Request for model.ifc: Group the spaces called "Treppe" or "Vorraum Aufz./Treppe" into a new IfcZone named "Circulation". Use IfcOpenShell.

First a look at what the model holds.

```python
import ifcopenshell

model = ifcopenshell.open("model.ifc")
print(model.schema)
seen = {}
for space in model.by_type("IfcSpace"):
    seen[space.LongName] = seen.get(space.LongName, 0) + 1
for name, count in sorted(seen.items(), key=str):
    print(count, "x", name)
print("zones:", [z.Name for z in model.by_type("IfcZone")][:20])
```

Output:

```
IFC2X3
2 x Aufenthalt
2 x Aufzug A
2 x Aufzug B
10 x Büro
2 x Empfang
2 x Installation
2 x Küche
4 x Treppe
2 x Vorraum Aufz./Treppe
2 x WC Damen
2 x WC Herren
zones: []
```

```python
import ifcopenshell
import ifcopenshell.api.group
import ifcopenshell.api.root

model = ifcopenshell.open("model.ifc")

names = {"Treppe", "Vorraum Aufz./Treppe"}
spaces = [s for s in model.by_type("IfcSpace") if s.LongName in names]

zone = ifcopenshell.api.root.create_entity(model, ifc_class="IfcZone", name="Circulation")
ifcopenshell.api.group.assign_group(model, products=spaces, group=zone)
print(len(spaces), "spaces in", zone.Name)

model.write("model_edited.ifc")
```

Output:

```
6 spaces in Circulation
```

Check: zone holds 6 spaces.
